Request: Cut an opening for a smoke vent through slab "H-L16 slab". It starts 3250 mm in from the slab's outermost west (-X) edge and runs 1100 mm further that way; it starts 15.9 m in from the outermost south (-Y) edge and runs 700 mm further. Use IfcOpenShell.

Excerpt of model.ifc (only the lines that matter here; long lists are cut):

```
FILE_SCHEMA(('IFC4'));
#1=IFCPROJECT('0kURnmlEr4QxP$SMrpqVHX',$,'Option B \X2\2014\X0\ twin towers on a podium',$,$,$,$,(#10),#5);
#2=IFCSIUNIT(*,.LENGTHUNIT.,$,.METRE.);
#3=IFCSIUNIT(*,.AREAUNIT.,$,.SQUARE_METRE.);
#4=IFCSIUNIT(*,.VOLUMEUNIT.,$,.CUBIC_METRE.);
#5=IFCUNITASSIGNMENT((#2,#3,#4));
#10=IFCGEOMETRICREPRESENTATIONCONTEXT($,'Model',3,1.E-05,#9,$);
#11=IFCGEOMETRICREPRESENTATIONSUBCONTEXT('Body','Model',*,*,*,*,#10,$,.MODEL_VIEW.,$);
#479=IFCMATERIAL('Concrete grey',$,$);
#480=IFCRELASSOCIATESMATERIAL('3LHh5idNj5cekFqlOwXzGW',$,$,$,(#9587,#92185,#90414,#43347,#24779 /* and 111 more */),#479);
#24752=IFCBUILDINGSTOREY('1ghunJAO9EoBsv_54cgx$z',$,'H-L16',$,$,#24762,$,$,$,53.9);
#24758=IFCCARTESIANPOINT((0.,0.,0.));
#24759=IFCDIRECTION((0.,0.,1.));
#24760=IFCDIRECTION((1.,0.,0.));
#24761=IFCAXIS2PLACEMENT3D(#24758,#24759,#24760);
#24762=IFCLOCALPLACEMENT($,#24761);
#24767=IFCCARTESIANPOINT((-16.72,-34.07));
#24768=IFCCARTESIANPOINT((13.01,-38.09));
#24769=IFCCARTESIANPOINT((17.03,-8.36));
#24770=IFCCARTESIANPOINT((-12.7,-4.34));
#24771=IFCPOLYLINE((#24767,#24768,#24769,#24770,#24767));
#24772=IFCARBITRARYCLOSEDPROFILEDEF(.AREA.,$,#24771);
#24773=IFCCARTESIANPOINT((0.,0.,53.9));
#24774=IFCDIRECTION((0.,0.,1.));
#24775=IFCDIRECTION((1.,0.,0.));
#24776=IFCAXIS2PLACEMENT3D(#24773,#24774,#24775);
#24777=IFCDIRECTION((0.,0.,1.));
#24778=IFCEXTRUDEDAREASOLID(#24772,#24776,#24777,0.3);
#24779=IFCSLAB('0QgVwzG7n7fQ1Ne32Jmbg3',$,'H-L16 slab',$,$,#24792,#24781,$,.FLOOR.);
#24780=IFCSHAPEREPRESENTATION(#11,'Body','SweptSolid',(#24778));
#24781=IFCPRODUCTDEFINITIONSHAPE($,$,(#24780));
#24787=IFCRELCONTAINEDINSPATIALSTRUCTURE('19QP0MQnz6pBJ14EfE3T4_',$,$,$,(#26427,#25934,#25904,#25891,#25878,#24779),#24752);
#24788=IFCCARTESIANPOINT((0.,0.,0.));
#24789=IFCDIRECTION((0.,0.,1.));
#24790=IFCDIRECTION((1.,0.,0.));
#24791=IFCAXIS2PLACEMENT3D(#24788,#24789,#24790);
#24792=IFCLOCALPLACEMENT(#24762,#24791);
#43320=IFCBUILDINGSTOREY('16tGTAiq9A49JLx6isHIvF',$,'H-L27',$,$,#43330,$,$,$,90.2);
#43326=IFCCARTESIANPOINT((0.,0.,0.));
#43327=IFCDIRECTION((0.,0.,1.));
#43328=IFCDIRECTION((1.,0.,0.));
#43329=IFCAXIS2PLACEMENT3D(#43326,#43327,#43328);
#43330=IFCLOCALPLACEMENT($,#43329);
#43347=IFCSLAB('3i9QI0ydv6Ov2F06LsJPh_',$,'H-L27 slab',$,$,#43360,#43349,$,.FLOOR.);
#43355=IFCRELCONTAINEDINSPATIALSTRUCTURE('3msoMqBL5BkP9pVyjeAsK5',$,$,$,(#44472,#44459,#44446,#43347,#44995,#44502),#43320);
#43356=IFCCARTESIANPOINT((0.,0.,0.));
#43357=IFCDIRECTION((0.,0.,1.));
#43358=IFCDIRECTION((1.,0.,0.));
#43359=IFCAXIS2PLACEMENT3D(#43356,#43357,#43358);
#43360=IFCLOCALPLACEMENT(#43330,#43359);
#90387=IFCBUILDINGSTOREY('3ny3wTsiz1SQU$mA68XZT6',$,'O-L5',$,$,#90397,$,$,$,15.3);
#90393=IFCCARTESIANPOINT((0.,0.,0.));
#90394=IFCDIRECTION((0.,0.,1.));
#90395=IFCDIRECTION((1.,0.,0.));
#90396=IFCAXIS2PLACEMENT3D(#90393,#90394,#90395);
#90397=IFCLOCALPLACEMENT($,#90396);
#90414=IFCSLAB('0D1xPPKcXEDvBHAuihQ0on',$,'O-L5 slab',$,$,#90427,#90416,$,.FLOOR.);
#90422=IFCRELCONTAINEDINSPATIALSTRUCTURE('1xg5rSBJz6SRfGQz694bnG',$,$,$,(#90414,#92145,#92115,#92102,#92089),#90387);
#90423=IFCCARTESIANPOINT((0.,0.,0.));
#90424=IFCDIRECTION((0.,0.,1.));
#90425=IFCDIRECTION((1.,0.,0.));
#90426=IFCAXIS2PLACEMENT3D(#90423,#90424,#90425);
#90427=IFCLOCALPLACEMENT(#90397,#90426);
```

```python
import numpy as np
import ifcopenshell
import ifcopenshell.api.feature
import ifcopenshell.api.geometry
import ifcopenshell.api.root
import ifcopenshell.geom
import ifcopenshell.util.placement
import ifcopenshell.util.representation
import ifcopenshell.util.shape
import ifcopenshell.util.unit

model = ifcopenshell.open("model.ifc")
unit_scale = ifcopenshell.util.unit.calculate_unit_scale(model)
settings = ifcopenshell.geom.settings()


def volume(element):
    """Net volume in cubic metres, openings subtracted."""
    shape = ifcopenshell.geom.create_shape(settings, element)
    return ifcopenshell.util.shape.get_volume(shape.geometry)


slab = model.by_id(24779)
before = volume(slab)

# Extent in the slab's own axes, in metres. The edges named are its -X and -Y sides.
slab_shape = ifcopenshell.geom.create_shape(settings, slab)
vertices = ifcopenshell.util.shape.get_vertices(slab_shape.geometry)
x_min, y_min, bottom = vertices.min(axis=0)
top = vertices[:, 2].max()

opening = ifcopenshell.api.root.create_entity(model, ifc_class="IfcOpeningElement", name="Smoke vent opening", predefined_type="OPENING")
context = ifcopenshell.util.representation.get_context(model, "Model", "Body", "MODEL_VIEW")
width, depth = 1.1, 0.7
outline = [(0.0, 0.0), (width, 0.0), (width, depth), (0.0, depth), (0.0, 0.0)]
# Overshoot both faces by 50 mm so the cut is clean.
shape = ifcopenshell.api.geometry.add_slab_representation(
    model, context=context, depth=top - bottom + 0.1, polyline=outline
)
ifcopenshell.api.geometry.assign_representation(model, product=opening, representation=shape)

matrix = ifcopenshell.util.placement.get_local_placement(slab.ObjectPlacement)
matrix[:, 3] = matrix @ np.append(np.array([x_min + 3.25, y_min + 15.9, bottom - 0.05]) / unit_scale, 1.0)
ifcopenshell.api.geometry.edit_object_placement(model, product=opening, matrix=matrix, is_si=False)
ifcopenshell.api.feature.add_feature(model, feature=opening, element=slab)

after = volume(slab)

print(f"slab volume {before:.3f} -> {after:.3f} m3")

model.write("model_rev.ifc")
```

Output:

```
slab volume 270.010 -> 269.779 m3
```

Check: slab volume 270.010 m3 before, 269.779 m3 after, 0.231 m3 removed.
